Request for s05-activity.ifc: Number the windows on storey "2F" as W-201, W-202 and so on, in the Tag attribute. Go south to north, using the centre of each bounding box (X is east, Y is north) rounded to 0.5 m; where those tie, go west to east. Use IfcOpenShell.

First a look at what the model holds.

```python
import ifcopenshell
import ifcopenshell.util.element
import ifcopenshell.util.placement

model = ifcopenshell.open("s05-activity.ifc")
print(model.schema)
storey = next(s for s in model.by_type("IfcBuildingStorey") if s.Name == "2F")
windows = [e for e in ifcopenshell.util.element.get_decomposition(storey) if e.is_a("IfcWindow")]
for e in sorted(windows, key=lambda e: e.id()):
    origin = ifcopenshell.util.placement.get_local_placement(e.ObjectPlacement)[:3, 3]
    print(e.id(), e.Tag, e.Name, origin.round(2) + 0.0, sep=" | ")
```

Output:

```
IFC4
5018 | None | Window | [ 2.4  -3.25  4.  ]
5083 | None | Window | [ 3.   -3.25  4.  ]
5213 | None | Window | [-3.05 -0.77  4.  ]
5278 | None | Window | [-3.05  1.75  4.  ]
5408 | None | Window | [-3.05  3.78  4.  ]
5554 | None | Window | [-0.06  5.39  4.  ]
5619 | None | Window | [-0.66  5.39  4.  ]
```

```python
import ifcopenshell
import ifcopenshell.geom
import ifcopenshell.util.element
import ifcopenshell.util.shape

model = ifcopenshell.open("s05-activity.ifc")
settings = ifcopenshell.geom.settings()
settings.set("use-world-coords", True)


def centre(element):
    shape = ifcopenshell.geom.create_shape(settings, element)
    return ifcopenshell.util.shape.get_bbox_centroid(shape.geometry)


storey = next(s for s in model.by_type("IfcBuildingStorey") if s.Name == "2F")
windows = [e for e in ifcopenshell.util.element.get_decomposition(storey) if e.is_a("IfcWindow")]

# Insertion points can sit at a corner or the storey origin, so sort by the geometry (in metres).
centres = {e: centre(e) for e in windows}
windows.sort(key=lambda e: (round(centres[e][1] / 0.5), centres[e][0]))

for i, e in enumerate(windows, start=1):
    number = f"W-2{i:02d}"
    e.Tag = number
    print(e.id(), number)

model.write("s05-activity_rev.ifc")
```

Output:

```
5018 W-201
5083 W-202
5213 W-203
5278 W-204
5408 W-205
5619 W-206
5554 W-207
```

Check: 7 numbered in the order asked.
